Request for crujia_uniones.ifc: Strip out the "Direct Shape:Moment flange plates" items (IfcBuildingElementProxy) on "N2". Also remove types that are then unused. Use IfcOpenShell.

First a look at what the model holds.

```python
import ifcopenshell
import ifcopenshell.util.element

model = ifcopenshell.open("crujia_uniones.ifc")
print(model.schema)
storey = next(s for s in model.by_type("IfcBuildingStorey") if s.Name == "N2")
proxies = [e for e in ifcopenshell.util.element.get_decomposition(storey) if e.is_a("IfcBuildingElementProxy")]
seen = {}
for e in proxies:
    element_type = ifcopenshell.util.element.get_type(e)
    name = element_type.Name if element_type not in (None, e) else None
    seen[name] = seen.get(name, 0) + 1
for name, count in sorted(seen.items(), key=str):
    print(count, "x", name)
```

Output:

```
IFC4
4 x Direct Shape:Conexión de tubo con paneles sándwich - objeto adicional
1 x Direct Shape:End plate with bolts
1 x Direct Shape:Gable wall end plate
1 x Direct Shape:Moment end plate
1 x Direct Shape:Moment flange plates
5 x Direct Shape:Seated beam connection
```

```python
import ifcopenshell
import ifcopenshell.api.root
import ifcopenshell.util.element

model = ifcopenshell.open("crujia_uniones.ifc")

storey = next(s for s in model.by_type("IfcBuildingStorey") if s.Name == "N2")
proxies = [e for e in ifcopenshell.util.element.get_decomposition(storey) if e.is_a("IfcBuildingElementProxy")]
targets = [e for e in proxies if (t := ifcopenshell.util.element.get_type(e)) not in (None, e) and t.Name == "Direct Shape:Moment flange plates"]
types = {ifcopenshell.util.element.get_type(e) for e in targets} - {None, *targets}

for e in targets:
    ifcopenshell.api.root.remove_product(model, product=e)
print(len(targets), "removed")

unused = [t for t in types if not ifcopenshell.util.element.get_types(t)]
for t in unused:
    ifcopenshell.api.root.remove_product(model, product=t)
print(len(unused), "unused types removed")

model.write("crujia_uniones_rev.ifc")
```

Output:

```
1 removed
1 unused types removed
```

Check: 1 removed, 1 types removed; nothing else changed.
